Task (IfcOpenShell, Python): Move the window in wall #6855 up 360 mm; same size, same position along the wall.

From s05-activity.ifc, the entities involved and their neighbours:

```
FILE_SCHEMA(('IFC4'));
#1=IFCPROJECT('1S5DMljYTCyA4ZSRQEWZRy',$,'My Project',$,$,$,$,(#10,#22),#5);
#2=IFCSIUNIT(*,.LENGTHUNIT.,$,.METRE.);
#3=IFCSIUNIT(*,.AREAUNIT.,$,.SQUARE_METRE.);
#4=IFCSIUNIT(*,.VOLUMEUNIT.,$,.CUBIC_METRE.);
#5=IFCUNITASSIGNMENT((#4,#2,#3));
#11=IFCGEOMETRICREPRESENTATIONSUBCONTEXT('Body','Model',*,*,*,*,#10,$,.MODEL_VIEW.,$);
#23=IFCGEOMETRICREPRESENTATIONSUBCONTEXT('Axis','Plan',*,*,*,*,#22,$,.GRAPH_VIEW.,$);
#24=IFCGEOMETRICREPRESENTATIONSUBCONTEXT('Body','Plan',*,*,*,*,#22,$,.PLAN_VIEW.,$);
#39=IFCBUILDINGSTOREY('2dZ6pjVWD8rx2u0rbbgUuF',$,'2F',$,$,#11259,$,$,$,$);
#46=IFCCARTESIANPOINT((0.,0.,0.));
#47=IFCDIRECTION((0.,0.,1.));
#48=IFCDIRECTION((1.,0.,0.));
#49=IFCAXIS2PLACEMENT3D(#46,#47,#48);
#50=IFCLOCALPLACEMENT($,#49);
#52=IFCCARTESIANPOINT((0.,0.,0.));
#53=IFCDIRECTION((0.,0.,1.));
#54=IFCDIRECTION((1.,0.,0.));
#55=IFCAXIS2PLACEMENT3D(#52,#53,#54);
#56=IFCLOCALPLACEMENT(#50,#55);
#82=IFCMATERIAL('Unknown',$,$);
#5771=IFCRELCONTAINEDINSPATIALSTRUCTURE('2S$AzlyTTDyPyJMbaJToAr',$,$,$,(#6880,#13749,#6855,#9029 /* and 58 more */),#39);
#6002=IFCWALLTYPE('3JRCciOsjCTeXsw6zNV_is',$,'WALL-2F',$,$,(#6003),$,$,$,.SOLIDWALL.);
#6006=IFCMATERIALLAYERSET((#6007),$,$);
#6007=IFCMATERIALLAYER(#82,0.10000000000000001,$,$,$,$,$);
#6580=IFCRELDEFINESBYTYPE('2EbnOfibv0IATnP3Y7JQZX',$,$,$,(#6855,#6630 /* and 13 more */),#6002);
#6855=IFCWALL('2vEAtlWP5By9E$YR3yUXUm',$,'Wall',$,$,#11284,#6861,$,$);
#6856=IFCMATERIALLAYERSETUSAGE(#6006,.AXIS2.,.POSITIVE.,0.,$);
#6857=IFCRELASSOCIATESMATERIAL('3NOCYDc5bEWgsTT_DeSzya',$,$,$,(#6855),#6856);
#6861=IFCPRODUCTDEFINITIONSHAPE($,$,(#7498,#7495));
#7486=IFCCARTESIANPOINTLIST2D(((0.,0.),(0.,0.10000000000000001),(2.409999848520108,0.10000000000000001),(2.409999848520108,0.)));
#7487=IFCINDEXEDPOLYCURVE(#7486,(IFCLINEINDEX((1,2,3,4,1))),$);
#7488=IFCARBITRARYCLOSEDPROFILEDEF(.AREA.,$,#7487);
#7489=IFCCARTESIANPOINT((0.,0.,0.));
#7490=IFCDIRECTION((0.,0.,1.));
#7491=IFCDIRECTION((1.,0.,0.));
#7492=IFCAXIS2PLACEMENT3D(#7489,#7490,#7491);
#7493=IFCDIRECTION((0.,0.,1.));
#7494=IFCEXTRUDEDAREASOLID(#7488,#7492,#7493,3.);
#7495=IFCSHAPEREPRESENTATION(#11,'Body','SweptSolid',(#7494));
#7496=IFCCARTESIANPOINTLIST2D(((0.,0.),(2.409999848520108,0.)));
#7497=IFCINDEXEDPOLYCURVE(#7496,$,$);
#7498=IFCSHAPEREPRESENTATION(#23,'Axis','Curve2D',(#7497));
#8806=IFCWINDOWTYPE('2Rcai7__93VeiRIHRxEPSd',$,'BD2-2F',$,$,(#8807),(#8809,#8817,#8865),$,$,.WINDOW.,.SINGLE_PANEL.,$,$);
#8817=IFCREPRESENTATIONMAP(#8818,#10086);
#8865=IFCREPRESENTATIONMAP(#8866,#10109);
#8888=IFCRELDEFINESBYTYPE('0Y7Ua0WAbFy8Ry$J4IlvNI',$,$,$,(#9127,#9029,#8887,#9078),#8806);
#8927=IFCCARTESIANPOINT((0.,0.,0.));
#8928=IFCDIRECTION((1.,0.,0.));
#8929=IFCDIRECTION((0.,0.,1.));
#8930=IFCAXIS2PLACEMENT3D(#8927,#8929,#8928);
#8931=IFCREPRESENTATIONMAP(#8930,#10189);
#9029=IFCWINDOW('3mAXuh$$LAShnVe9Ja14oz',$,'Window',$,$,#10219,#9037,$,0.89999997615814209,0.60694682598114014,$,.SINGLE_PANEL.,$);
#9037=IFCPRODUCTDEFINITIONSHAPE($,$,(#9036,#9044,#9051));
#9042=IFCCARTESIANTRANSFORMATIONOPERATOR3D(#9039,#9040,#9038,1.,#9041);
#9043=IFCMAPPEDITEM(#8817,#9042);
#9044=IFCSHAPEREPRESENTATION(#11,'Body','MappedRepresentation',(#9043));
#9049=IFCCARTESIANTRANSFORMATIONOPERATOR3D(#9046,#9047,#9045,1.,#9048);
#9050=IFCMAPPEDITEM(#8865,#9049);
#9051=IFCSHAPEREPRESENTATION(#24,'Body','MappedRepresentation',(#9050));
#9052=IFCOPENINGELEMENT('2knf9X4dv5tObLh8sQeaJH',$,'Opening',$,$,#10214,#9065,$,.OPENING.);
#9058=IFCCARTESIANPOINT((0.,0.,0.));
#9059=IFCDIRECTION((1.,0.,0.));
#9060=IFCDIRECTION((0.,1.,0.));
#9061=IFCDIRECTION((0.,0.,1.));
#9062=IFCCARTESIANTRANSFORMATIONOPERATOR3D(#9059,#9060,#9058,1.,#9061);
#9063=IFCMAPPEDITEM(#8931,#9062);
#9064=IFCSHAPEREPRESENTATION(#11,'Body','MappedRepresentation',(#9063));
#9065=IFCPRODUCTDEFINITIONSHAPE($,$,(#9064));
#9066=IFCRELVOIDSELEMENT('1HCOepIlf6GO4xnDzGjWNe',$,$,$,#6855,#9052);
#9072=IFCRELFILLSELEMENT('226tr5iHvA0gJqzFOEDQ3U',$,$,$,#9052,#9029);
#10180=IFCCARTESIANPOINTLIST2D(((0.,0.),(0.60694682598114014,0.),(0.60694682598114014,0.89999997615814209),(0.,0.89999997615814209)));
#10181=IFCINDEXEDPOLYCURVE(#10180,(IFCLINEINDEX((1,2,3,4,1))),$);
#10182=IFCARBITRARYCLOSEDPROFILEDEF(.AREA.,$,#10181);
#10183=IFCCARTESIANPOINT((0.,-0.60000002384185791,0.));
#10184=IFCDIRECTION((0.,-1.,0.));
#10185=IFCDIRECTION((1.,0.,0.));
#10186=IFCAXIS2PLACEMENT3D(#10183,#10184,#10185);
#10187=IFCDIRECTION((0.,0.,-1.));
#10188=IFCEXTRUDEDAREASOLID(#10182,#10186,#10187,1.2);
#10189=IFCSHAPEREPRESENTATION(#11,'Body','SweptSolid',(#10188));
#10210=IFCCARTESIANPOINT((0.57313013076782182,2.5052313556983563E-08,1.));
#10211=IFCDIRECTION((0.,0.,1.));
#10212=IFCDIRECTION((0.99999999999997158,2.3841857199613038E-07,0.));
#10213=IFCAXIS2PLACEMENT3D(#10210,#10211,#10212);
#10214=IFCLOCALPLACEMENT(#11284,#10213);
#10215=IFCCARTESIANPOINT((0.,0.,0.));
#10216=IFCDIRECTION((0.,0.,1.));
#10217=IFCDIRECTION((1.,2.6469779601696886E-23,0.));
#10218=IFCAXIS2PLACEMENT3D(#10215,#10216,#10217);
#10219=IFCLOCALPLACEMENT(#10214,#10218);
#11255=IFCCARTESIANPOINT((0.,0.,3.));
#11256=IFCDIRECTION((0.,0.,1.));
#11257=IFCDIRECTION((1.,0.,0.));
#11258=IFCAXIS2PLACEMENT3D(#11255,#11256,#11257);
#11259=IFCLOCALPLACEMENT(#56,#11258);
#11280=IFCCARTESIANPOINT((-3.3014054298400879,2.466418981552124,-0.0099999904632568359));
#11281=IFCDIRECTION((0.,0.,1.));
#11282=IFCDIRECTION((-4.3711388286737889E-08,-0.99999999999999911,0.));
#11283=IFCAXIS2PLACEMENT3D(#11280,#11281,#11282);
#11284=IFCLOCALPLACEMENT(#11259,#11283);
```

```python
import numpy as np
import ifcopenshell
import ifcopenshell.api.geometry
import ifcopenshell.util.placement
import ifcopenshell.util.unit

model = ifcopenshell.open("s05-activity.ifc")
unit_scale = ifcopenshell.util.unit.calculate_unit_scale(model)

window = model.by_guid("3mAXuh$$LAShnVe9Ja14oz")
opening = window.FillsVoids[0].RelatingOpeningElement
dz = 0.36

shift = np.array([0.0, 0.0, dz])
# The window is placed relative to its opening, so it follows when the opening moves.
matrix = ifcopenshell.util.placement.get_local_placement(opening.ObjectPlacement)
matrix[:3, 3] += shift
ifcopenshell.api.geometry.edit_object_placement(
    model, product=opening, matrix=matrix, is_si=False, should_transform_children=True
)

print(f"moved by {dz * unit_scale:+.3f} m")

model.write("s05-activity_rev.ifc")
```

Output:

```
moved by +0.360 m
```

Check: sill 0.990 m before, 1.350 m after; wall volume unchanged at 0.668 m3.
